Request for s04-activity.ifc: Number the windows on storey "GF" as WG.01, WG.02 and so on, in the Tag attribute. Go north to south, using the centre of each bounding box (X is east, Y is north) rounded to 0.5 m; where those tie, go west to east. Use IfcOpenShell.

First a look at what the model holds.

```python
import ifcopenshell
import ifcopenshell.util.element
import ifcopenshell.util.placement

model = ifcopenshell.open("s04-activity.ifc")
print(model.schema)
storey = next(s for s in model.by_type("IfcBuildingStorey") if s.Name == "GF")
windows = [e for e in ifcopenshell.util.element.get_decomposition(storey) if e.is_a("IfcWindow")]
for e in sorted(windows, key=lambda e: e.id()):
    origin = ifcopenshell.util.placement.get_local_placement(e.ObjectPlacement)[:3, 3]
    print(e.id(), e.Tag, e.Name, origin.round(2) + 0.0, sep=" | ")
```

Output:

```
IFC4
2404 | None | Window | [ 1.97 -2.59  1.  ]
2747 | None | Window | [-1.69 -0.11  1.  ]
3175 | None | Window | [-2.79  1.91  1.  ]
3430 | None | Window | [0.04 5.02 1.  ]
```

```python
import ifcopenshell
import ifcopenshell.geom
import ifcopenshell.util.element
import ifcopenshell.util.shape

model = ifcopenshell.open("s04-activity.ifc")
settings = ifcopenshell.geom.settings()
settings.set("use-world-coords", True)


def centre(element):
    shape = ifcopenshell.geom.create_shape(settings, element)
    return ifcopenshell.util.shape.get_bbox_centroid(shape.geometry)


storey = next(s for s in model.by_type("IfcBuildingStorey") if s.Name == "GF")
windows = [e for e in ifcopenshell.util.element.get_decomposition(storey) if e.is_a("IfcWindow")]

# Insertion points can sit at a corner or the storey origin, so sort by the geometry (in metres).
centres = {e: centre(e) for e in windows}
windows.sort(key=lambda e: (-round(centres[e][1] / 0.5), centres[e][0]))

for i, e in enumerate(windows, start=1):
    number = f"WG.{i:02d}"
    e.Tag = number
    print(e.id(), number)

model.write("s04-activity_rev.ifc")
```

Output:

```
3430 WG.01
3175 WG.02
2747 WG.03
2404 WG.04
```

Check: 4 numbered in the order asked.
